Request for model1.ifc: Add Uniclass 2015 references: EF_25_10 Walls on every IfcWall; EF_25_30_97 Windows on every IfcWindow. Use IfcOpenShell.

First a look at what the model holds.

```python
import ifcopenshell

model = ifcopenshell.open("model1.ifc")
print(model.schema)
print("classifications:", [c.Name for c in model.by_type("IfcClassification")])
for ifc_class in ("IfcDoor", "IfcRoof", "IfcStair", "IfcWall", "IfcWindow"):
    print(ifc_class, len(model.by_type(ifc_class)))
```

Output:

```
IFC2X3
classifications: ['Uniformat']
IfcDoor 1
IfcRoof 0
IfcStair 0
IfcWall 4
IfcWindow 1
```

```python
import ifcopenshell
import ifcopenshell.api.classification

model = ifcopenshell.open("model1.ifc")

# IFC2X3 requires Source and Edition and has no link from the project to the system.
system = model.create_entity("IfcClassification", Source="NBS", Edition="2015", Name="Uniclass 2015")

codes = {
    "IfcWall": ("EF_25_10", "Walls"),
    "IfcWindow": ("EF_25_30_97", "Windows"),
}
for ifc_class, (code, name) in codes.items():
    products = model.by_type(ifc_class)
    ifcopenshell.api.classification.add_reference(
        model, products=products, classification=system, identification=code, name=name
    )
    print(code, len(products))

model.write("model1_v2.ifc")
```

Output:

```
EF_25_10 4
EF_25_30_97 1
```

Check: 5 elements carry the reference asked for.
